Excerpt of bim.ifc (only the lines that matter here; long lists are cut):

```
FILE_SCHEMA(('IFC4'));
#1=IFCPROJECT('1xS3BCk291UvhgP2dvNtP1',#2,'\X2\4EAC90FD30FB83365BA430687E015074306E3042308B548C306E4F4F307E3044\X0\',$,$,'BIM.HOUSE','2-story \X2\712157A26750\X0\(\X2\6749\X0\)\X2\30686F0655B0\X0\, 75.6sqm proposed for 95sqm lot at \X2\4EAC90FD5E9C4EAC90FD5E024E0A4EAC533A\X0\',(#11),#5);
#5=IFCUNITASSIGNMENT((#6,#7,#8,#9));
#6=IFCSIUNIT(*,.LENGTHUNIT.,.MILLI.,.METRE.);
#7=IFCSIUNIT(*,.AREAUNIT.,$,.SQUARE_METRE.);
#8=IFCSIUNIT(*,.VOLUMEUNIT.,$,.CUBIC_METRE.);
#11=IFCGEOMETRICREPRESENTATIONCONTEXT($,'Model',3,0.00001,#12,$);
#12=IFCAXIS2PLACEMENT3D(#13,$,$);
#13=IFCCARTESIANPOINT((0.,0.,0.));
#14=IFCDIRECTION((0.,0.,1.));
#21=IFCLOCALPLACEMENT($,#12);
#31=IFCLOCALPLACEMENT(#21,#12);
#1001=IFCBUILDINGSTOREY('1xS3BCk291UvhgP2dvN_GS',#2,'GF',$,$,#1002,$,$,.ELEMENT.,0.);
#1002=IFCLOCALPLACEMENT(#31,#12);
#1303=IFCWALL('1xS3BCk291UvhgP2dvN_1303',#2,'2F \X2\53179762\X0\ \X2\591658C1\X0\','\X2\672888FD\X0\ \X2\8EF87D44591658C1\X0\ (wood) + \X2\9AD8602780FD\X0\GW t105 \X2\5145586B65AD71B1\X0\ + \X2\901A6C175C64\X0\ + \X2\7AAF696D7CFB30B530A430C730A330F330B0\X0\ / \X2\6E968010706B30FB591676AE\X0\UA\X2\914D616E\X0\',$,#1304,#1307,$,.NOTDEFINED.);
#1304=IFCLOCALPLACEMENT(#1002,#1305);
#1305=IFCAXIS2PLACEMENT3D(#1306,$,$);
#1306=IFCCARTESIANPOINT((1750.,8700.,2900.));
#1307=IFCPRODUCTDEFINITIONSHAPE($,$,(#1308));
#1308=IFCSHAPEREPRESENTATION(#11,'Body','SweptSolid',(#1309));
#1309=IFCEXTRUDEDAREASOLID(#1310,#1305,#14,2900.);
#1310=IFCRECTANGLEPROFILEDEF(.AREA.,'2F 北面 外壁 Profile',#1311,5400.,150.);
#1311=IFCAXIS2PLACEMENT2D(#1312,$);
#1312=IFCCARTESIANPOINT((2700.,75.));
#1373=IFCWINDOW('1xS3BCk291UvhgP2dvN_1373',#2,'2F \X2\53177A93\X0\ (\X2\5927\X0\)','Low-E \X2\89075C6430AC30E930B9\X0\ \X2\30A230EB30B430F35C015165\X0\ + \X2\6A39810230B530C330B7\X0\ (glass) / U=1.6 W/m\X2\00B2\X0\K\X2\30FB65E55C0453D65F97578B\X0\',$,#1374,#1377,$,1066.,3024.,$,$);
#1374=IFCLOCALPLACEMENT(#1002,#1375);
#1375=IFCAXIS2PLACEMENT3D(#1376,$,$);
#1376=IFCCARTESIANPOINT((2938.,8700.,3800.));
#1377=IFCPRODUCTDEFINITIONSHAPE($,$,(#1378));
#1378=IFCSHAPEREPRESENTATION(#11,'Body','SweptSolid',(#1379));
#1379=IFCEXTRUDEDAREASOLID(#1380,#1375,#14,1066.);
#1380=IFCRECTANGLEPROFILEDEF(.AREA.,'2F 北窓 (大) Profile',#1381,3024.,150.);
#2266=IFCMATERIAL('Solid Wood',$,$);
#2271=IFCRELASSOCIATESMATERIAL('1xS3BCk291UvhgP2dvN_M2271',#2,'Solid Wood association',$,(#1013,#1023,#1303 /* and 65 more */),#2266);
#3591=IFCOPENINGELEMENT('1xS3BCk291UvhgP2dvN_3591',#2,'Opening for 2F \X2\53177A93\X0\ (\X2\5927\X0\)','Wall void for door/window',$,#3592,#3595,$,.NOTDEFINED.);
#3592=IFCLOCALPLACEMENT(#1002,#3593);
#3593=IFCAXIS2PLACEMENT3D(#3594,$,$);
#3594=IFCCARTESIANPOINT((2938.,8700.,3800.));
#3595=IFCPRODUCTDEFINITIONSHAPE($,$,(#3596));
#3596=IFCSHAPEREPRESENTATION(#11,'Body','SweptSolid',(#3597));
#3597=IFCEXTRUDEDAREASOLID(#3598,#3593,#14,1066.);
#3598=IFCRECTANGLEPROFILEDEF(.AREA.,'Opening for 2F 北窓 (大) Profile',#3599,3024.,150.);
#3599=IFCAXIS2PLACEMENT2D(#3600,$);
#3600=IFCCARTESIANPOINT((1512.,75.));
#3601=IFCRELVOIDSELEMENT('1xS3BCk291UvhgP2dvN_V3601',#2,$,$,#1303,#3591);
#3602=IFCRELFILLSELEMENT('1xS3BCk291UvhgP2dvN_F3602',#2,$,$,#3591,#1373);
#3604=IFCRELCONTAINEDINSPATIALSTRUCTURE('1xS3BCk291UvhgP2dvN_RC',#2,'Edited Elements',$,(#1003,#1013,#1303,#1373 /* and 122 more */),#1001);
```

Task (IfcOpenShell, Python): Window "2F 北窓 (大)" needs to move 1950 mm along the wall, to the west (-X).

```python
import ifcopenshell
import ifcopenshell.api.geometry
import ifcopenshell.util.placement

model = ifcopenshell.open("bim.ifc")

window = model.by_guid("1xS3BCk291UvhgP2dvN_1373")
opening = window.FillsVoids[0].RelatingOpeningElement
wall = opening.VoidsElements[0].RelatingBuildingElement

wall_matrix = ifcopenshell.util.placement.get_local_placement(wall.ObjectPlacement)
shift = wall_matrix[:3, 0] * -1950.0
before = ifcopenshell.util.placement.get_local_placement(window.ObjectPlacement)[:3, 3].copy()

# The window is not placed relative to its opening, so move both.
for product in (opening, window):
    matrix = ifcopenshell.util.placement.get_local_placement(product.ObjectPlacement)
    matrix[:3, 3] += shift
    ifcopenshell.api.geometry.edit_object_placement(model, product=product, matrix=matrix, is_si=False)

after = ifcopenshell.util.placement.get_local_placement(window.ObjectPlacement)[:3, 3]
print("window moved by", (after - before).round(3) + 0.0)

model.write("bim_edited.ifc")
```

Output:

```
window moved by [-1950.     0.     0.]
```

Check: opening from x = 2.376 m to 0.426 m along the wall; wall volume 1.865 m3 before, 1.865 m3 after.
